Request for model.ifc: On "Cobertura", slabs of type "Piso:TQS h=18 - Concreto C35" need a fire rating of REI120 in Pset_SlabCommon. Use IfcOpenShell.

First a look at what the model holds.

```python
import ifcopenshell
import ifcopenshell.util.element

model = ifcopenshell.open("model.ifc")
print(model.schema)
storey = next(s for s in model.by_type("IfcBuildingStorey") if s.Name == "Cobertura")
slabs = [e for e in ifcopenshell.util.element.get_decomposition(storey) if e.is_a("IfcSlab")]
seen = {}
for e in slabs:
    element_type = ifcopenshell.util.element.get_type(e)
    key = (element_type.Name if element_type != e and element_type else None, ifcopenshell.util.element.get_pset(e, "Pset_SlabCommon", "FireRating"))
    seen[key] = seen.get(key, 0) + 1
for (name, value), count in sorted(seen.items(), key=str):
    print(count, "x", name, "|", value)
```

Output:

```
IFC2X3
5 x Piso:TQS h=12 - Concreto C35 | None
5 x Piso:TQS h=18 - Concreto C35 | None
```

```python
import ifcopenshell
import ifcopenshell.api.pset
import ifcopenshell.util.element

model = ifcopenshell.open("model.ifc")

storey = next(s for s in model.by_type("IfcBuildingStorey") if s.Name == "Cobertura")
slabs = [e for e in ifcopenshell.util.element.get_decomposition(storey) if e.is_a("IfcSlab")]

count = 0
for e in slabs:
    element_type = ifcopenshell.util.element.get_type(e)
    if element_type in (None, e) or element_type.Name != "Piso:TQS h=18 - Concreto C35":
        continue
    # add_pset returns the element's existing set when there is one.
    pset = ifcopenshell.api.pset.add_pset(model, product=e, name="Pset_SlabCommon")
    ifcopenshell.api.pset.edit_pset(model, pset=pset, properties={"FireRating": "REI120"})
    count += 1

print(count, "slabs updated")

model.write("model_updated.ifc")
```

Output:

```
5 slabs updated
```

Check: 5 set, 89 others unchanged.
